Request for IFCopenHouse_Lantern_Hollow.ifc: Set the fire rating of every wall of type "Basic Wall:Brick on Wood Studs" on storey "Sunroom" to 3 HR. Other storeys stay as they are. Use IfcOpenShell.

First a look at what the model holds.

```python
import ifcopenshell
import ifcopenshell.util.element

model = ifcopenshell.open("IFCopenHouse_Lantern_Hollow.ifc")
print(model.schema)
storey = next(s for s in model.by_type("IfcBuildingStorey") if s.Name == "Sunroom")
walls = [e for e in ifcopenshell.util.element.get_decomposition(storey) if e.is_a("IfcWall")]
seen = {}
for e in walls:
    element_type = ifcopenshell.util.element.get_type(e)
    key = (element_type.Name if element_type != e and element_type else None, ifcopenshell.util.element.get_pset(e, "Pset_WallCommon", "FireRating"))
    seen[key] = seen.get(key, 0) + 1
for (name, value), count in sorted(seen.items(), key=str):
    print(count, "x", name, "|", value)
```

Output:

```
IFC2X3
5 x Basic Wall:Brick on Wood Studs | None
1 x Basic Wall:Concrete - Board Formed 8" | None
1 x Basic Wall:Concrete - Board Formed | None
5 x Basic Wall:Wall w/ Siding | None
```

```python
import ifcopenshell
import ifcopenshell.api.pset
import ifcopenshell.util.element

model = ifcopenshell.open("IFCopenHouse_Lantern_Hollow.ifc")

storey = next(s for s in model.by_type("IfcBuildingStorey") if s.Name == "Sunroom")
walls = [e for e in ifcopenshell.util.element.get_decomposition(storey) if e.is_a("IfcWall")]

count = 0
for e in walls:
    element_type = ifcopenshell.util.element.get_type(e)
    if element_type in (None, e) or element_type.Name != "Basic Wall:Brick on Wood Studs":
        continue
    # add_pset returns the element's existing set when there is one.
    pset = ifcopenshell.api.pset.add_pset(model, product=e, name="Pset_WallCommon")
    ifcopenshell.api.pset.edit_pset(model, pset=pset, properties={"FireRating": "3 HR"})
    count += 1

print(count, "walls updated")

model.write("IFCopenHouse_Lantern_Hollow-out.ifc")
```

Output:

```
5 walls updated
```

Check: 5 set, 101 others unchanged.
